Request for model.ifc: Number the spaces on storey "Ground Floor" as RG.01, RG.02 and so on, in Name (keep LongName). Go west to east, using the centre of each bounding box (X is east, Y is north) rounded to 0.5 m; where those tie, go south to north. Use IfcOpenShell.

First a look at what the model holds.

```python
import ifcopenshell
import ifcopenshell.util.element
import ifcopenshell.util.placement

model = ifcopenshell.open("model.ifc")
print(model.schema)
storey = next(s for s in model.by_type("IfcBuildingStorey") if s.Name == "Ground Floor")
spaces = [e for e in ifcopenshell.util.element.get_decomposition(storey) if e.is_a("IfcSpace")]
for e in sorted(spaces, key=lambda e: e.id()):
    origin = ifcopenshell.util.placement.get_local_placement(e.ObjectPlacement)[:3, 3]
    print(e.id(), e.Name, e.LongName, origin.round(2) + 0.0, sep=" | ")
```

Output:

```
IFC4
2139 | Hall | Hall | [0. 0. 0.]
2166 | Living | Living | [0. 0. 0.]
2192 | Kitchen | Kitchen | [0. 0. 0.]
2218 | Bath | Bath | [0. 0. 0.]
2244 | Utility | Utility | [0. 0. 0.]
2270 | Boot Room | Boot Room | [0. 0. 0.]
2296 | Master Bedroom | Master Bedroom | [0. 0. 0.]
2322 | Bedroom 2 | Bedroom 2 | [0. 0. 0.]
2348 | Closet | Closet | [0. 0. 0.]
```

```python
import ifcopenshell
import ifcopenshell.geom
import ifcopenshell.util.element
import ifcopenshell.util.shape

model = ifcopenshell.open("model.ifc")
settings = ifcopenshell.geom.settings()
settings.set("use-world-coords", True)


def centre(element):
    shape = ifcopenshell.geom.create_shape(settings, element)
    return ifcopenshell.util.shape.get_bbox_centroid(shape.geometry)


storey = next(s for s in model.by_type("IfcBuildingStorey") if s.Name == "Ground Floor")
spaces = [e for e in ifcopenshell.util.element.get_decomposition(storey) if e.is_a("IfcSpace")]

# Insertion points can sit at a corner or the storey origin, so sort by the geometry (in metres).
centres = {e: centre(e) for e in spaces}
spaces.sort(key=lambda e: (round(centres[e][0] / 0.5), centres[e][1]))

for i, e in enumerate(spaces, start=1):
    number = f"RG.{i:02d}"
    e.Name = number
    print(e.id(), number)

model.write("model-out.ifc")
```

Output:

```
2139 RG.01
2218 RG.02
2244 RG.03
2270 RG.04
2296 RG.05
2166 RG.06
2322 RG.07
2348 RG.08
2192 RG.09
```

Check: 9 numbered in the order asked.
